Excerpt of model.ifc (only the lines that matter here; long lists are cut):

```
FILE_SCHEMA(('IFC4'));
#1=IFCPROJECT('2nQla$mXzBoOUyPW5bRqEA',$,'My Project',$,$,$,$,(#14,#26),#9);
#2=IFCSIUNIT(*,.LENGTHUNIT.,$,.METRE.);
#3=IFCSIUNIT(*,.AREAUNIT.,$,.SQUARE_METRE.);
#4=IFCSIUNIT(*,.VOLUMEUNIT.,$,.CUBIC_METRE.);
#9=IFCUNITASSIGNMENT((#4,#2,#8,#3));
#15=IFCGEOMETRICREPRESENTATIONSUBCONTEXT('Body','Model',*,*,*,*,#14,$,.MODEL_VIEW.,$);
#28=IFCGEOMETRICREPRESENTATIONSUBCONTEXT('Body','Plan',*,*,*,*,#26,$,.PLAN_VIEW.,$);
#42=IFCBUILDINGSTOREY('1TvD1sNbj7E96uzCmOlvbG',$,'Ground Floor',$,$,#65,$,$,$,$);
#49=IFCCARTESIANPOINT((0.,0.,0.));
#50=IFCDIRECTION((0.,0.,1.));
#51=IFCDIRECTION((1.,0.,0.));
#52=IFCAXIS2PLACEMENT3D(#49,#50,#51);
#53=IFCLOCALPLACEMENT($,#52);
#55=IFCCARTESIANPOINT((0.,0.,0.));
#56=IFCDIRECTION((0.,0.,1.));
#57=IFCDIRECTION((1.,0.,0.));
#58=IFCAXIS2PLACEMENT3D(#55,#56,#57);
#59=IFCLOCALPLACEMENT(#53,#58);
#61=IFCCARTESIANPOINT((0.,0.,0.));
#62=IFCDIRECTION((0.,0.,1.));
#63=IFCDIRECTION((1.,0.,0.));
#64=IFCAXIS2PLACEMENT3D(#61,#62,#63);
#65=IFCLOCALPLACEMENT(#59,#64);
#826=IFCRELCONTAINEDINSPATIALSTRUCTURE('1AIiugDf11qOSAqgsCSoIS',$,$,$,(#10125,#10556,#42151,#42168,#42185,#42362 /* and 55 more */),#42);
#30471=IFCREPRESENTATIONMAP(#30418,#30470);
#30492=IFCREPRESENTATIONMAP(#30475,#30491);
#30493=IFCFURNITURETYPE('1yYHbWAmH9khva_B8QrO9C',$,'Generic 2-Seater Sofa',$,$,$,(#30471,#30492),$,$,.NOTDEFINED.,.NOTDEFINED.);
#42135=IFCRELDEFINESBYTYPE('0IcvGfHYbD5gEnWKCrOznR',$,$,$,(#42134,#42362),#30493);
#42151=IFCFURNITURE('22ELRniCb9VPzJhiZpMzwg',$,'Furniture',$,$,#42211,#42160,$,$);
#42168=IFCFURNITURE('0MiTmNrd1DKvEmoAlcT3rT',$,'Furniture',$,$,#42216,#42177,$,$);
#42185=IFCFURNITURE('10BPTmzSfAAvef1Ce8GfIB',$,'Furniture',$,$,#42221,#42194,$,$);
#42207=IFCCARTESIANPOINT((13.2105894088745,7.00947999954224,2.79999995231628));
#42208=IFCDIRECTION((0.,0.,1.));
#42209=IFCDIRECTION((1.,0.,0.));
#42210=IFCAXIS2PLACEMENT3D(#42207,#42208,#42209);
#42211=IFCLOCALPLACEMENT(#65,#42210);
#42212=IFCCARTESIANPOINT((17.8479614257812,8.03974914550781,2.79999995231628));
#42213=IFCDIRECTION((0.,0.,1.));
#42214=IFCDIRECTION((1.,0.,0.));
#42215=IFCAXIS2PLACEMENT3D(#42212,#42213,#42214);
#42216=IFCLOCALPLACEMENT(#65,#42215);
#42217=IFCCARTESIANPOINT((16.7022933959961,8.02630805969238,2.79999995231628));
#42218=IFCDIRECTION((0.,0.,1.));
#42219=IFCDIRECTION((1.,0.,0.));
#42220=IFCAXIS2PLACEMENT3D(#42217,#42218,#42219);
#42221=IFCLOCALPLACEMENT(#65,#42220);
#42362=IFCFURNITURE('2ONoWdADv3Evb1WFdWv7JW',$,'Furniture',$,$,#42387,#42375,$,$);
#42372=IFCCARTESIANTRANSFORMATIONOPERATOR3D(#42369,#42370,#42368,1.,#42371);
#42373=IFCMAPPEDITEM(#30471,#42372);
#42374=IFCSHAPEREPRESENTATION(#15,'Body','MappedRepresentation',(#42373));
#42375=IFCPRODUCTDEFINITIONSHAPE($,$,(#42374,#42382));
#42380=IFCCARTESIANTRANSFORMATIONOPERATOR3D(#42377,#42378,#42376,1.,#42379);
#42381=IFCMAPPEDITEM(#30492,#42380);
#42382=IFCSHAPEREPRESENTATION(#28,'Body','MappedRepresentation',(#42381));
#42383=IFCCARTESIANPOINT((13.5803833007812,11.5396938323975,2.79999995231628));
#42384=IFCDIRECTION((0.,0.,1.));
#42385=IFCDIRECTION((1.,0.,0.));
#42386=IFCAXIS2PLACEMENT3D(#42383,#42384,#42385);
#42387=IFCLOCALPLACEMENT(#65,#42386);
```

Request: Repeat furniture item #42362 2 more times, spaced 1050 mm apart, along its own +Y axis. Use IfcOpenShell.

```python
import ifcopenshell
import ifcopenshell.api.geometry
import ifcopenshell.api.root
import ifcopenshell.util.element
import ifcopenshell.util.placement

model = ifcopenshell.open("model.ifc")

source = model.by_guid("2ONoWdADv3Evb1WFdWv7JW")
base = ifcopenshell.util.placement.get_local_placement(source.ObjectPlacement)
step = base[:3, 1] * 1.05

for i in range(1, 3):
    copy = ifcopenshell.api.root.copy_class(model, product=source)
    copy.Representation = ifcopenshell.util.element.copy_deep(
        model, source.Representation, exclude=["IfcGeometricRepresentationContext", "IfcRepresentationMap"]
    )
    matrix = base.copy()
    matrix[:3, 3] += i * step
    print("added at", matrix[:3, 3].round(3) + 0.0)
    ifcopenshell.api.geometry.edit_object_placement(model, product=copy, matrix=matrix, is_si=False)

model.write("model-out.ifc")
```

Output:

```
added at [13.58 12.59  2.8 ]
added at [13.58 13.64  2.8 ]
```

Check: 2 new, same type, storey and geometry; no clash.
